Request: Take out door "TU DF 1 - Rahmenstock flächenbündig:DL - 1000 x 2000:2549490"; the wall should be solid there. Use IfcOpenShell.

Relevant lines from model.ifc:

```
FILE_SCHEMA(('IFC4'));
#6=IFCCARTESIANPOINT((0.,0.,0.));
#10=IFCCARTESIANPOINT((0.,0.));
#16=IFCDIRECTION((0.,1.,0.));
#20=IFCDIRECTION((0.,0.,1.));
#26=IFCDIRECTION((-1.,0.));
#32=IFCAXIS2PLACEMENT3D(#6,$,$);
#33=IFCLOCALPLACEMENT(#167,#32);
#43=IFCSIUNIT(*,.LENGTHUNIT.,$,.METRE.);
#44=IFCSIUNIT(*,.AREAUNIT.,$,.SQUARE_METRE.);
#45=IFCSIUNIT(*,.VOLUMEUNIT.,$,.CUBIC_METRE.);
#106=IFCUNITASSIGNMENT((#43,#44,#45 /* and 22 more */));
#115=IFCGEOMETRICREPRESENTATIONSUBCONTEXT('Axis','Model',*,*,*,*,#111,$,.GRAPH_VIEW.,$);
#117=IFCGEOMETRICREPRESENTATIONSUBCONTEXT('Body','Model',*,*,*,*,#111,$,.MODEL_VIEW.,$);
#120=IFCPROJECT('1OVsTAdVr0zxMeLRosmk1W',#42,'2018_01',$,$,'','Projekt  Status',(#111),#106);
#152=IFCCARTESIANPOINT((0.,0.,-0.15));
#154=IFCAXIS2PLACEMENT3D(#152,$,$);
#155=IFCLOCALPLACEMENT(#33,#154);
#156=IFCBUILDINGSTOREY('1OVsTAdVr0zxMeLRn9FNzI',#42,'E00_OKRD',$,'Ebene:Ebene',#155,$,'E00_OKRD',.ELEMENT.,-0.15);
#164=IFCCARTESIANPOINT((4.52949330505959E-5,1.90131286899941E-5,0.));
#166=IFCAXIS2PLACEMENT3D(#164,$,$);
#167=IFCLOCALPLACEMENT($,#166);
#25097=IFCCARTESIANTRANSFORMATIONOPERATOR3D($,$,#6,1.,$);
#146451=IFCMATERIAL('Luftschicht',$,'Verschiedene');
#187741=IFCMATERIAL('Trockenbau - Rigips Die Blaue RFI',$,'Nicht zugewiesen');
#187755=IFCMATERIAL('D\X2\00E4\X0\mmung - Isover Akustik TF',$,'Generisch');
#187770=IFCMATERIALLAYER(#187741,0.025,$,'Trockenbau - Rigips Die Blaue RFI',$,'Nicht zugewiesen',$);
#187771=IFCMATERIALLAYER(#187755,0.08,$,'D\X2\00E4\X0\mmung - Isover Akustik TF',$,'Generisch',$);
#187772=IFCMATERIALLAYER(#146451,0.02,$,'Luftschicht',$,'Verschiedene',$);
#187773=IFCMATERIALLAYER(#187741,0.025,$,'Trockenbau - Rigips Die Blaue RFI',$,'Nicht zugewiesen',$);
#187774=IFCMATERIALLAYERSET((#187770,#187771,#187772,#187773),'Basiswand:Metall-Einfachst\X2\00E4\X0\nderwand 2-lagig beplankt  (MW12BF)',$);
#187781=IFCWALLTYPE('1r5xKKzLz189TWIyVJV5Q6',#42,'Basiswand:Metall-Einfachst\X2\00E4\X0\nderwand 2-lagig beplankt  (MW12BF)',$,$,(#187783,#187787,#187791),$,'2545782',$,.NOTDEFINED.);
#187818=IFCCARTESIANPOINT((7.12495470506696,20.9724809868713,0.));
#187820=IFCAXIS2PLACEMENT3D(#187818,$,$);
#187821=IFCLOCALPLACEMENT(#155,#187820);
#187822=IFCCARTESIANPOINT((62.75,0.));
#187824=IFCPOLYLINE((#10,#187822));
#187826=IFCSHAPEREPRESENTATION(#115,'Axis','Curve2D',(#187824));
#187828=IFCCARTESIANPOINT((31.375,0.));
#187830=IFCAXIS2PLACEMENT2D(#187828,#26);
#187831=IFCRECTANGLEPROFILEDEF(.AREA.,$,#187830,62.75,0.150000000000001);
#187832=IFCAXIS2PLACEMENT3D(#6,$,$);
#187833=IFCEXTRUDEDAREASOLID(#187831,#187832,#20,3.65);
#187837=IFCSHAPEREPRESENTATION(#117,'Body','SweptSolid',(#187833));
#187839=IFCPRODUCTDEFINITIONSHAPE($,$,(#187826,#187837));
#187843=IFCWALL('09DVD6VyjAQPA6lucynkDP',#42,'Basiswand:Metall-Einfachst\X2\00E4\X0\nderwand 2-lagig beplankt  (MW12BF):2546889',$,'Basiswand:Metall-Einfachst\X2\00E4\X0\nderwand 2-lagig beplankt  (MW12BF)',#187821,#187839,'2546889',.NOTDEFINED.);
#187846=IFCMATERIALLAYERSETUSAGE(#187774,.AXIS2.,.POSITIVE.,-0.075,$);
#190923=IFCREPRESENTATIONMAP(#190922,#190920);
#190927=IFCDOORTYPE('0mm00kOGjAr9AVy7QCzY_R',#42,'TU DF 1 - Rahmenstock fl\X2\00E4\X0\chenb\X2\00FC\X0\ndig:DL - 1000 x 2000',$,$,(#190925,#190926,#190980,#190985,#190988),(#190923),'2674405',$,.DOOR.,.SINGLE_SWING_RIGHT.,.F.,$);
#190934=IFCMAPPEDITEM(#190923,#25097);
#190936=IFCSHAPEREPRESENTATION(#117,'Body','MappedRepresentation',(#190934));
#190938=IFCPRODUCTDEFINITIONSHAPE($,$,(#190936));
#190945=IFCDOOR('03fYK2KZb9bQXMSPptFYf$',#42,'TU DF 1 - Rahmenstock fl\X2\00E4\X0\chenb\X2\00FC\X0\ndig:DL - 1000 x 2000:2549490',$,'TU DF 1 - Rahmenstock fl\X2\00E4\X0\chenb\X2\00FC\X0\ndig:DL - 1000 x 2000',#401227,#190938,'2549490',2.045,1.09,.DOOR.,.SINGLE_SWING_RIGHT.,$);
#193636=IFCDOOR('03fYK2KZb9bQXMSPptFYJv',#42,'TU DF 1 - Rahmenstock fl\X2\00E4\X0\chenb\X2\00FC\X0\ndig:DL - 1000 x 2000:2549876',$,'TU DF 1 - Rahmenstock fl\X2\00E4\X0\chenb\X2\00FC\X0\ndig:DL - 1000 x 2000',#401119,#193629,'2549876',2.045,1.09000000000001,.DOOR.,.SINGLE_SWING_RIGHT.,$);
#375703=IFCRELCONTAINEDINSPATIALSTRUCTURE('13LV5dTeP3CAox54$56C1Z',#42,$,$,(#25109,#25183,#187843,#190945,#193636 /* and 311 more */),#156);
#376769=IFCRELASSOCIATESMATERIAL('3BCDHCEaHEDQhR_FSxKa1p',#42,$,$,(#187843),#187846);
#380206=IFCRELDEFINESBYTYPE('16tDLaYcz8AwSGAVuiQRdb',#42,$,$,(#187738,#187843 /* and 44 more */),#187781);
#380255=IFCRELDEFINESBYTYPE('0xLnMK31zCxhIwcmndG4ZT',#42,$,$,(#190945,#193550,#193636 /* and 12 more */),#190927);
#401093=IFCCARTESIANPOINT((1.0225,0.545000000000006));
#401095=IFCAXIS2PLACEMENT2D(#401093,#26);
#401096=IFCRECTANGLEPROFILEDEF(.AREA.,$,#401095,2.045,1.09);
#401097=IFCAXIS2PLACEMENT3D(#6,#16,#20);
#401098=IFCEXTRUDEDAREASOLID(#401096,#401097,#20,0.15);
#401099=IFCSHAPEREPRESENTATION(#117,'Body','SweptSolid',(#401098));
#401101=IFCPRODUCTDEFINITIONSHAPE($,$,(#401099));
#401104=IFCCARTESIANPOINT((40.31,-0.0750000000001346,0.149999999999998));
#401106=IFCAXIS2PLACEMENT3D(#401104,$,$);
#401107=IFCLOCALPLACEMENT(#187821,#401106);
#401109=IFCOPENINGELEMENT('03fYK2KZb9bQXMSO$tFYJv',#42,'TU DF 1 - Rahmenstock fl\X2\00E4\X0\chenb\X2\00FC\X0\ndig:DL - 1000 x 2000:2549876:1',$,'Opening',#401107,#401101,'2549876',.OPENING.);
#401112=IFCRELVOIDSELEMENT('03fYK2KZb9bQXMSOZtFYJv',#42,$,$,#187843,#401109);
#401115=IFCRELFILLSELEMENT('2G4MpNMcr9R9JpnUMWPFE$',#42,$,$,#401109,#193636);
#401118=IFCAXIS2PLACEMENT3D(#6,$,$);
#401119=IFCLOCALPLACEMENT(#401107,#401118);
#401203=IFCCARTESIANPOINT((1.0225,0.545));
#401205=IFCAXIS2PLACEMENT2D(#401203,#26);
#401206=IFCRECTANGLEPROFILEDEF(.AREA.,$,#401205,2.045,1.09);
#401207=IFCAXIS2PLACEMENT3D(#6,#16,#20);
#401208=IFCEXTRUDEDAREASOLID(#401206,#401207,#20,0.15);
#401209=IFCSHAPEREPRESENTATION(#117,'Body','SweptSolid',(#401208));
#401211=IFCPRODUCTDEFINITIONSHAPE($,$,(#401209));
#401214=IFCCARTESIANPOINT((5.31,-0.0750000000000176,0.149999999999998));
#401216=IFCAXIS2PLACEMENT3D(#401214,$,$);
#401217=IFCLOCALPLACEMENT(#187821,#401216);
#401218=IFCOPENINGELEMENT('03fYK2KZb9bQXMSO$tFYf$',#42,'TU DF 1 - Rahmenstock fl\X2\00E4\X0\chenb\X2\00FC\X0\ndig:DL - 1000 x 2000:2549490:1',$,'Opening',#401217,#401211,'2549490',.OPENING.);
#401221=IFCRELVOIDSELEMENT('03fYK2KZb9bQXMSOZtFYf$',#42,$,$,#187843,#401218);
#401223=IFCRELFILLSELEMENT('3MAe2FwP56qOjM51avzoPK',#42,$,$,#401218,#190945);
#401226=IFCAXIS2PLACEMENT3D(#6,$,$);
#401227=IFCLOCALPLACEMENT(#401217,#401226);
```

```python
import ifcopenshell
import ifcopenshell.api.feature
import ifcopenshell.api.root
import ifcopenshell.geom
import ifcopenshell.util.shape

model = ifcopenshell.open("model.ifc")
settings = ifcopenshell.geom.settings()


def volume(element):
    """Net volume in cubic metres, openings subtracted."""
    shape = ifcopenshell.geom.create_shape(settings, element)
    return ifcopenshell.util.shape.get_volume(shape.geometry)


door = model.by_guid("03fYK2KZb9bQXMSPptFYf$")
opening = door.FillsVoids[0].RelatingOpeningElement
wall = opening.VoidsElements[0].RelatingBuildingElement
before = volume(wall)

ifcopenshell.api.root.remove_product(model, product=door)
ifcopenshell.api.feature.remove_feature(model, feature=opening)

after = volume(wall)

print(f"wall volume {before:.3f} -> {after:.3f} m3")

model.write("model-out.ifc")
```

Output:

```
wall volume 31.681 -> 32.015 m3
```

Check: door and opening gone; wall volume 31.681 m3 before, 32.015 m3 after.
